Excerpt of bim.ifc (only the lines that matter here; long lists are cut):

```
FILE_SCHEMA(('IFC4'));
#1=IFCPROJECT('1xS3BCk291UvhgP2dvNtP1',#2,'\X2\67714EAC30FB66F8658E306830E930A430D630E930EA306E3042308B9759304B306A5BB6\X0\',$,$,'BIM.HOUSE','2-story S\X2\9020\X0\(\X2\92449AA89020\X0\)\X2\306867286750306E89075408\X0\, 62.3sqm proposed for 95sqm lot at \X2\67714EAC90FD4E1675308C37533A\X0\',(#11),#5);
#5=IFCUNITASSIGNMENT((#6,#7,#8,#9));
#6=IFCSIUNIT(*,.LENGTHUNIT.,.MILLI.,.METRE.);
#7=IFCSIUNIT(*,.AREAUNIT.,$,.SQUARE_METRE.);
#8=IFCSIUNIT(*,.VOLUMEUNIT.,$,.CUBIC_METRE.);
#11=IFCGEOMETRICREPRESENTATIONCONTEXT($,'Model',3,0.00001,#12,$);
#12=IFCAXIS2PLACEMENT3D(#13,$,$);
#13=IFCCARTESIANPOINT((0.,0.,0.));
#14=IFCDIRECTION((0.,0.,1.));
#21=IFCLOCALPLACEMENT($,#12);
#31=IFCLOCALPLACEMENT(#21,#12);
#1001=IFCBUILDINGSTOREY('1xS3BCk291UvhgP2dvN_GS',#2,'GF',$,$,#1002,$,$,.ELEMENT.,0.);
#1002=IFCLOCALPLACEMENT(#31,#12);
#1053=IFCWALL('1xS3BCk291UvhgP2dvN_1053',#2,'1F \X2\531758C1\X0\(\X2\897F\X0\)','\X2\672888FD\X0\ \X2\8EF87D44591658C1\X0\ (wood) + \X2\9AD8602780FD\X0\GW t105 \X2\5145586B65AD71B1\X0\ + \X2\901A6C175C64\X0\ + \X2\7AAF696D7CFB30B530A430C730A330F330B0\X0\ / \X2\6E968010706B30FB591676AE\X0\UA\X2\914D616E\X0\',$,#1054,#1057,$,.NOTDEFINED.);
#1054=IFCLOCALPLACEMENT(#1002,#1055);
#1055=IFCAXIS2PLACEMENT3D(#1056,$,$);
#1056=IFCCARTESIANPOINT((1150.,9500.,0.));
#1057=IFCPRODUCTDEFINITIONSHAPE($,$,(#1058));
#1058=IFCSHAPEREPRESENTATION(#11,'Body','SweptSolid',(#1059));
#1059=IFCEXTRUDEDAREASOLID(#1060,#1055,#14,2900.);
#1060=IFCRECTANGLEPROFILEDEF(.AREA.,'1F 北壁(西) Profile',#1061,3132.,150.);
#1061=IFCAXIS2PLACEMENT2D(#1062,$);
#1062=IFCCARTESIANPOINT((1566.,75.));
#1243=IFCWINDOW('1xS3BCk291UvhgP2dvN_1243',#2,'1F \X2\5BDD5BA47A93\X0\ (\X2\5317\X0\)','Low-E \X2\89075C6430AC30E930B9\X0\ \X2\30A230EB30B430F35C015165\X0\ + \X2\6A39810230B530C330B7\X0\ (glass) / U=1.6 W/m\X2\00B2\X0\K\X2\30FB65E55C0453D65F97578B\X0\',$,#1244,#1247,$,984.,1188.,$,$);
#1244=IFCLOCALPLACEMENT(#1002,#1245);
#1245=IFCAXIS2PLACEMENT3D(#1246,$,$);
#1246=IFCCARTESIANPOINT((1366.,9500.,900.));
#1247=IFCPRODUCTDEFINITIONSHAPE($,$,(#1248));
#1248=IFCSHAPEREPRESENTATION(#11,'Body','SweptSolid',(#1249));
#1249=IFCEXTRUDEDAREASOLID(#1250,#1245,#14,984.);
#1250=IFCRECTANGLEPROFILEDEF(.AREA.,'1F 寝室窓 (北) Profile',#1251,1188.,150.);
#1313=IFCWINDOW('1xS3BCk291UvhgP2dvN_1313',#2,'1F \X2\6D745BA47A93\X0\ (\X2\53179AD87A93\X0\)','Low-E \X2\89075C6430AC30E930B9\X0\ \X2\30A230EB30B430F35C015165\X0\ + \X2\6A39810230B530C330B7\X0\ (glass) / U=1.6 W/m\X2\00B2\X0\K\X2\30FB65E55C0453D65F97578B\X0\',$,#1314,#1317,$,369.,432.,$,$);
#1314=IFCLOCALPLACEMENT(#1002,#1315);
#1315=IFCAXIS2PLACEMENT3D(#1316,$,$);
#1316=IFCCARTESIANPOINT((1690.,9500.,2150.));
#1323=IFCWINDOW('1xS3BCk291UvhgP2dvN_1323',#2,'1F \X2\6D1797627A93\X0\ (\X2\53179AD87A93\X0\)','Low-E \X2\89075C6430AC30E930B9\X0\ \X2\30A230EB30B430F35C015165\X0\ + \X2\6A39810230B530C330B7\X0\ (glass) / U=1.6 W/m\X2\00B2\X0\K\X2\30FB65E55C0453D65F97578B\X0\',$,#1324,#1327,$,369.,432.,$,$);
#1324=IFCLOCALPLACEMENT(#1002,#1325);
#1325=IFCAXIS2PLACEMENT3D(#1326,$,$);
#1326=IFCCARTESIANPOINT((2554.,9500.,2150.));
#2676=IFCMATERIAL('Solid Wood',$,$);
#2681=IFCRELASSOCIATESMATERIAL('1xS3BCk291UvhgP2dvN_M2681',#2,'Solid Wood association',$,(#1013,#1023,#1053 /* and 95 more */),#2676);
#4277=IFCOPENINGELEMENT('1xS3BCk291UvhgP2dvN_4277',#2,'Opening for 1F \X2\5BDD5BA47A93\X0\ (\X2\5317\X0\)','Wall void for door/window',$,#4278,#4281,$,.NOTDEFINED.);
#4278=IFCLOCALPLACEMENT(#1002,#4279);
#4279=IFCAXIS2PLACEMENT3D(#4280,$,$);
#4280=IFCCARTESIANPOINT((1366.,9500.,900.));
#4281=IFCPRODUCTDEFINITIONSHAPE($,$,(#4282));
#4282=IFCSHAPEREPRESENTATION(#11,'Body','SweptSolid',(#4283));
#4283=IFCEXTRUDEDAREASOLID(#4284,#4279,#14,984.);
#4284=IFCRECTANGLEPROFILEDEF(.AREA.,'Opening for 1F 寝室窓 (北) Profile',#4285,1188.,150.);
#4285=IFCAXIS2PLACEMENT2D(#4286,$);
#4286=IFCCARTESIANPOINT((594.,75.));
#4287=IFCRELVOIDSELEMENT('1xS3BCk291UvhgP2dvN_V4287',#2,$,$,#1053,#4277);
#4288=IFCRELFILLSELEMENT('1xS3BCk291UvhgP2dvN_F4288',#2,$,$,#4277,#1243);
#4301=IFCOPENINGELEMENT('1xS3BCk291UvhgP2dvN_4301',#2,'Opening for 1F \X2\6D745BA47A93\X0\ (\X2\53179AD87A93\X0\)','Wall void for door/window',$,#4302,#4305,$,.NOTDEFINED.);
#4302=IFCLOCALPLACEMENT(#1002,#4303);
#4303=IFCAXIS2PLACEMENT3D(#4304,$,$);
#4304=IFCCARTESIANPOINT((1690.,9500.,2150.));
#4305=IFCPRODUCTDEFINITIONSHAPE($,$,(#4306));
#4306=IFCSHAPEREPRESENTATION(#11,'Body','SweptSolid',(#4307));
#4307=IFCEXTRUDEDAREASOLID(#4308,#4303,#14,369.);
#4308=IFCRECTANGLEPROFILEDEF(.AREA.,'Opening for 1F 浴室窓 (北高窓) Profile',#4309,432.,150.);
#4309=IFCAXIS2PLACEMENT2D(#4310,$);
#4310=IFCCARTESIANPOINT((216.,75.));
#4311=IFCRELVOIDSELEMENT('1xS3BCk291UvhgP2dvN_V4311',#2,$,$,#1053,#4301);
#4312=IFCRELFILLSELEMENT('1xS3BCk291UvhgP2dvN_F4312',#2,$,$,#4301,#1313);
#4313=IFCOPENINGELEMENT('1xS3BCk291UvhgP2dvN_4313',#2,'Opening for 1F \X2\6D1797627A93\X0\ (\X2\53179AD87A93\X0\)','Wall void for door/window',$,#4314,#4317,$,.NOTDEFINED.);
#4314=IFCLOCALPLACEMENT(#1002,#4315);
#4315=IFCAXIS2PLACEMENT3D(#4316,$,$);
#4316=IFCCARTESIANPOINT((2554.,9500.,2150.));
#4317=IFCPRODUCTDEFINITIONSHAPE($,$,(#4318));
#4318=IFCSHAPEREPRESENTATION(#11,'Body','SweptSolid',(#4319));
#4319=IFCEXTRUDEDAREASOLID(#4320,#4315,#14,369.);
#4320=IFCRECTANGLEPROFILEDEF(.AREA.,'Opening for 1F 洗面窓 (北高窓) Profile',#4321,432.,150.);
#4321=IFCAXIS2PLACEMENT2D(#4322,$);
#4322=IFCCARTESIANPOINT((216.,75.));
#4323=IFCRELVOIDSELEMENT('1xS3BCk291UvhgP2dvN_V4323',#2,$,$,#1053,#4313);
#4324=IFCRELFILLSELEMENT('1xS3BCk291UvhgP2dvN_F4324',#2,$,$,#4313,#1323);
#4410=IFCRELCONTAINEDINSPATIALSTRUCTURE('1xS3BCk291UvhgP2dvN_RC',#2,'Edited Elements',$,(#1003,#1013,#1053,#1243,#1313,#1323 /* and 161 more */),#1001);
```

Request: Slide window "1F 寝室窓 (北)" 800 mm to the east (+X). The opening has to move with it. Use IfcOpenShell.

```python
import ifcopenshell
import ifcopenshell.api.geometry
import ifcopenshell.util.placement
import ifcopenshell.util.unit

model = ifcopenshell.open("bim.ifc")
unit_scale = ifcopenshell.util.unit.calculate_unit_scale(model)

window = model.by_id(1243)
opening = window.FillsVoids[0].RelatingOpeningElement
wall = opening.VoidsElements[0].RelatingBuildingElement

wall_matrix = ifcopenshell.util.placement.get_local_placement(wall.ObjectPlacement)
shift = wall_matrix[:3, 0] * 0.8 / unit_scale
before = ifcopenshell.util.placement.get_local_placement(window.ObjectPlacement)[:3, 3].copy()

# The window is not placed relative to its opening, so move both.
for product in (opening, window):
    matrix = ifcopenshell.util.placement.get_local_placement(product.ObjectPlacement)
    matrix[:3, 3] += shift
    ifcopenshell.api.geometry.edit_object_placement(model, product=product, matrix=matrix, is_si=False)

after = ifcopenshell.util.placement.get_local_placement(window.ObjectPlacement)[:3, 3]
print("window moved by", (after - before).round(3) + 0.0)

model.write("bim_v2.ifc")
```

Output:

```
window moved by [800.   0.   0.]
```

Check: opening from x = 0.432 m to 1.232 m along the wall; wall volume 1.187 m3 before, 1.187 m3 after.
